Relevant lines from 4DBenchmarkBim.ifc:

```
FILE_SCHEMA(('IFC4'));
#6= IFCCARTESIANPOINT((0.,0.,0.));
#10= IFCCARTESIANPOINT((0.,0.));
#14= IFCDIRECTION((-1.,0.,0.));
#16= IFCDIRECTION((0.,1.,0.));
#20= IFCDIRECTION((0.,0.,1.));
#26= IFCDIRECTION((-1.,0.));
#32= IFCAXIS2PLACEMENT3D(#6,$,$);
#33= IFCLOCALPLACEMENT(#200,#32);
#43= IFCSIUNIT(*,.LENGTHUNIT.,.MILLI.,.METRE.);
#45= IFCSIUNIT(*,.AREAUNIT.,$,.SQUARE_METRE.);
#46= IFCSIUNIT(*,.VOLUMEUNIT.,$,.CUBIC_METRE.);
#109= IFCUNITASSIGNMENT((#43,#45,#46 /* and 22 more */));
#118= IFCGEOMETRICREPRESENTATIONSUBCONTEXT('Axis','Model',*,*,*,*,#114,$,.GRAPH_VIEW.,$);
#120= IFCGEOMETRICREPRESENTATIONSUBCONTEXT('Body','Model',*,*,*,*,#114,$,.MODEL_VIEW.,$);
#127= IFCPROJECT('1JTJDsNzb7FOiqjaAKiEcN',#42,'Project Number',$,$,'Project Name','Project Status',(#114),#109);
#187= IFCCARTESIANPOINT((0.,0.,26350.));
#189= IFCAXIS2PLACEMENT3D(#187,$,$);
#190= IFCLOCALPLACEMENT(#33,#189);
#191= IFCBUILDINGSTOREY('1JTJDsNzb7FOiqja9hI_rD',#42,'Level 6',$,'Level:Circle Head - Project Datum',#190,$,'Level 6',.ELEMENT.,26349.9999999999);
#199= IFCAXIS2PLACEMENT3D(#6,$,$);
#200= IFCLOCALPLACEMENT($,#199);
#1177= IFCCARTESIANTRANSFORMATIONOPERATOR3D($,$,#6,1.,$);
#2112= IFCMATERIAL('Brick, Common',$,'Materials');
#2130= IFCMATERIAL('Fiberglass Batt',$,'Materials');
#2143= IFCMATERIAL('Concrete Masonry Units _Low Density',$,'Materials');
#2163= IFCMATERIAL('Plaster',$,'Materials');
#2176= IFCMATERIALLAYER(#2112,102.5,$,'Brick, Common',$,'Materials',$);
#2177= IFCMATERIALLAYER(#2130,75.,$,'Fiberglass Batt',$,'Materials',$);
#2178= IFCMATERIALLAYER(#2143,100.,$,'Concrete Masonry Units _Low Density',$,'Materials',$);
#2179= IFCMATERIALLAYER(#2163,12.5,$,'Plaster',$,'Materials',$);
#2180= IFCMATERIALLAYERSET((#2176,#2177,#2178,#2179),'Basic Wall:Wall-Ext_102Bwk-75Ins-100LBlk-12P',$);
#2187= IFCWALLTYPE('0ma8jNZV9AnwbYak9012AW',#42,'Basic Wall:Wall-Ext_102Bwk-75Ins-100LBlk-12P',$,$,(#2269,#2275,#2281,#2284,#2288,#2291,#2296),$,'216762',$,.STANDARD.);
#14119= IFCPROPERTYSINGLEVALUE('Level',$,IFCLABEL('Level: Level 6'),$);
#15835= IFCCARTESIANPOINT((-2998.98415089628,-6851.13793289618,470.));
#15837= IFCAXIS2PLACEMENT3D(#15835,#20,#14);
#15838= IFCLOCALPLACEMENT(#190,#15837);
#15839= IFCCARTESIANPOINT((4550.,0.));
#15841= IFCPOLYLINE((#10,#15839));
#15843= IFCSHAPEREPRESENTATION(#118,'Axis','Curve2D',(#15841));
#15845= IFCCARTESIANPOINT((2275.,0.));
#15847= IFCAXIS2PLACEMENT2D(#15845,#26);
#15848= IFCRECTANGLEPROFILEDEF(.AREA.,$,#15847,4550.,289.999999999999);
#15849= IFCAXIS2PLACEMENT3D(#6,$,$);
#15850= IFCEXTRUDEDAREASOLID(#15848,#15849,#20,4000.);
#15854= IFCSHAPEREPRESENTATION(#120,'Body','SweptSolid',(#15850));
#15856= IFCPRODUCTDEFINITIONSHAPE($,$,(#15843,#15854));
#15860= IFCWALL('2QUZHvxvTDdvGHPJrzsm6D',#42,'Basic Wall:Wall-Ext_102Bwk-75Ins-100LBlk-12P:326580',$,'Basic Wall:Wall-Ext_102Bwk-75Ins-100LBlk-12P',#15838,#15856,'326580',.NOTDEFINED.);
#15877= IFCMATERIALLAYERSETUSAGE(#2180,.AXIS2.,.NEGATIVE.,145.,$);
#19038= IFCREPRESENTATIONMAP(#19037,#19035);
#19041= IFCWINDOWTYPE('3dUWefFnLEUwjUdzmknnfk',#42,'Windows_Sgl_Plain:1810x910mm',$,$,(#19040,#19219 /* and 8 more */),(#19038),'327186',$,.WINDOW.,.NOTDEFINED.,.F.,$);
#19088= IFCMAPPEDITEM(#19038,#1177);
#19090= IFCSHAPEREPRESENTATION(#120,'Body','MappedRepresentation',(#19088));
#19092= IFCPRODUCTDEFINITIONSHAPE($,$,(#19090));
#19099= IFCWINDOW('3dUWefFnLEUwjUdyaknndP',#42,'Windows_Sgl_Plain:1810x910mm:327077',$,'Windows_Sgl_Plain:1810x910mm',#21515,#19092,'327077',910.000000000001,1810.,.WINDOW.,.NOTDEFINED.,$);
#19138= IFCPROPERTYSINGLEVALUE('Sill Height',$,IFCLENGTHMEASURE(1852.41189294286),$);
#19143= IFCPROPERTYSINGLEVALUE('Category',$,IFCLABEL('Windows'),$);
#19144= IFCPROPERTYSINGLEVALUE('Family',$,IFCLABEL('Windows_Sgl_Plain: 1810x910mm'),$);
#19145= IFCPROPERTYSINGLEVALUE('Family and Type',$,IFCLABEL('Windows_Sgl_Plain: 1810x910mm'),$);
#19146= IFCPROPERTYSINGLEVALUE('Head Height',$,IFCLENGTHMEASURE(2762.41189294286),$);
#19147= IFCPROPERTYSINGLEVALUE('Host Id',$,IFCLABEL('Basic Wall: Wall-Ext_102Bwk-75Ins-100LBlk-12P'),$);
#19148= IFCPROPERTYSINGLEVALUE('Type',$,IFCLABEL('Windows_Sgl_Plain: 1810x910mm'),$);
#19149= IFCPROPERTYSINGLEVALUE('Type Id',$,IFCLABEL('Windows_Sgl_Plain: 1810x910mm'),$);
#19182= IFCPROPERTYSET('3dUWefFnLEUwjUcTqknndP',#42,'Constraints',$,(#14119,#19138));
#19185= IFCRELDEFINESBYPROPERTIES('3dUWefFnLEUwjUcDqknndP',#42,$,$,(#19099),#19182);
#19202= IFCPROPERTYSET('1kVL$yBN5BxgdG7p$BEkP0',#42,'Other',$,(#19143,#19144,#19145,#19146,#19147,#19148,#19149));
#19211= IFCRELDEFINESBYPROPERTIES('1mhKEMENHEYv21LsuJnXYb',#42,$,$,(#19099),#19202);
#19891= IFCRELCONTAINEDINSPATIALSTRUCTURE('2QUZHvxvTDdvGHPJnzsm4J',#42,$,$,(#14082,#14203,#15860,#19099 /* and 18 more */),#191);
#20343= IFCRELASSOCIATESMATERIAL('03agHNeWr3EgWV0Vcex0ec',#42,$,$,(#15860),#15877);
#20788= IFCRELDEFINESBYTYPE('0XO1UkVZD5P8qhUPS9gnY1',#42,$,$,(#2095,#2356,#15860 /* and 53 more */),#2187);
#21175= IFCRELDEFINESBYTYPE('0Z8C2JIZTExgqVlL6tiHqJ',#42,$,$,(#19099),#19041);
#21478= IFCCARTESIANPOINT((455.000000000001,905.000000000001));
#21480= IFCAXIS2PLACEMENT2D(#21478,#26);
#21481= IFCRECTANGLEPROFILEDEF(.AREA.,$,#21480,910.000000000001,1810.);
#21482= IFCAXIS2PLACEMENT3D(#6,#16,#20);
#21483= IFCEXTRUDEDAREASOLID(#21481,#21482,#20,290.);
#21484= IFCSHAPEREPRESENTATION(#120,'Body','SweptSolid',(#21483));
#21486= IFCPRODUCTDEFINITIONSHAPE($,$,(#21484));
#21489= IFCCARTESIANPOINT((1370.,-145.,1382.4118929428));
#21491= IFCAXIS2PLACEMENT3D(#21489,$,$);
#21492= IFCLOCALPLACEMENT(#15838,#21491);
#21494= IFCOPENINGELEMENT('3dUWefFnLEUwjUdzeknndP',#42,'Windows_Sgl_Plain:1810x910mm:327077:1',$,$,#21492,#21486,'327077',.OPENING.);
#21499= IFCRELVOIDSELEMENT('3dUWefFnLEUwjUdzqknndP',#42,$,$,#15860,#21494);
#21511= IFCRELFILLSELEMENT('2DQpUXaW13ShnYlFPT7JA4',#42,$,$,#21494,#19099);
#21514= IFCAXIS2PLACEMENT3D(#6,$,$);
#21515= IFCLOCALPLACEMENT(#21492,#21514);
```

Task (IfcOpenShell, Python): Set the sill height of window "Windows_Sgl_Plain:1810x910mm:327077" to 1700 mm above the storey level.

```python
import numpy as np
import ifcopenshell
import ifcopenshell.api.geometry
import ifcopenshell.api.pset
import ifcopenshell.geom
import ifcopenshell.util.element
import ifcopenshell.util.placement
import ifcopenshell.util.shape
import ifcopenshell.util.unit

model = ifcopenshell.open("4DBenchmarkBim.ifc")
unit_scale = ifcopenshell.util.unit.calculate_unit_scale(model)

window = model.by_guid("3dUWefFnLEUwjUdyaknndP")
opening = window.FillsVoids[0].RelatingOpeningElement
storey = ifcopenshell.util.element.get_container(window, ifc_class="IfcBuildingStorey")
level = ifcopenshell.util.placement.get_local_placement(storey.ObjectPlacement)[2, 3]

# The opening's origin need not be at the sill, so measure its lowest point.
shape = ifcopenshell.geom.create_shape(ifcopenshell.geom.settings(), opening)
bottom = ifcopenshell.util.shape.get_shape_bottom_elevation(shape, shape.geometry) / unit_scale
dz = level + 1700.0 - bottom

shift = np.array([0.0, 0.0, dz])
# The window is placed relative to its opening, so it follows when the opening moves.
matrix = ifcopenshell.util.placement.get_local_placement(opening.ObjectPlacement)
matrix[:3, 3] += shift
ifcopenshell.api.geometry.edit_object_placement(
    model, product=opening, matrix=matrix, is_si=False, should_transform_children=True
)

# Keep the stored heights in step.
pset = model.by_id(ifcopenshell.util.element.get_pset(window, "Constraints", should_inherit=False)["id"])
ifcopenshell.api.pset.edit_pset(model, pset=pset, properties={
    "Sill Height": model.create_entity("IfcLengthMeasure", ifcopenshell.util.element.get_pset(window, "Constraints", "Sill Height") + dz),
})
pset = model.by_id(ifcopenshell.util.element.get_pset(window, "Other", should_inherit=False)["id"])
ifcopenshell.api.pset.edit_pset(model, pset=pset, properties={
    "Head Height": model.create_entity("IfcLengthMeasure", ifcopenshell.util.element.get_pset(window, "Other", "Head Height") + dz),
})

print(f"moved by {dz * unit_scale:+.3f} m")

model.write("4DBenchmarkBim_rev.ifc")
```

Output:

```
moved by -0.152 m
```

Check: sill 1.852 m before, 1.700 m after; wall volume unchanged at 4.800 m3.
